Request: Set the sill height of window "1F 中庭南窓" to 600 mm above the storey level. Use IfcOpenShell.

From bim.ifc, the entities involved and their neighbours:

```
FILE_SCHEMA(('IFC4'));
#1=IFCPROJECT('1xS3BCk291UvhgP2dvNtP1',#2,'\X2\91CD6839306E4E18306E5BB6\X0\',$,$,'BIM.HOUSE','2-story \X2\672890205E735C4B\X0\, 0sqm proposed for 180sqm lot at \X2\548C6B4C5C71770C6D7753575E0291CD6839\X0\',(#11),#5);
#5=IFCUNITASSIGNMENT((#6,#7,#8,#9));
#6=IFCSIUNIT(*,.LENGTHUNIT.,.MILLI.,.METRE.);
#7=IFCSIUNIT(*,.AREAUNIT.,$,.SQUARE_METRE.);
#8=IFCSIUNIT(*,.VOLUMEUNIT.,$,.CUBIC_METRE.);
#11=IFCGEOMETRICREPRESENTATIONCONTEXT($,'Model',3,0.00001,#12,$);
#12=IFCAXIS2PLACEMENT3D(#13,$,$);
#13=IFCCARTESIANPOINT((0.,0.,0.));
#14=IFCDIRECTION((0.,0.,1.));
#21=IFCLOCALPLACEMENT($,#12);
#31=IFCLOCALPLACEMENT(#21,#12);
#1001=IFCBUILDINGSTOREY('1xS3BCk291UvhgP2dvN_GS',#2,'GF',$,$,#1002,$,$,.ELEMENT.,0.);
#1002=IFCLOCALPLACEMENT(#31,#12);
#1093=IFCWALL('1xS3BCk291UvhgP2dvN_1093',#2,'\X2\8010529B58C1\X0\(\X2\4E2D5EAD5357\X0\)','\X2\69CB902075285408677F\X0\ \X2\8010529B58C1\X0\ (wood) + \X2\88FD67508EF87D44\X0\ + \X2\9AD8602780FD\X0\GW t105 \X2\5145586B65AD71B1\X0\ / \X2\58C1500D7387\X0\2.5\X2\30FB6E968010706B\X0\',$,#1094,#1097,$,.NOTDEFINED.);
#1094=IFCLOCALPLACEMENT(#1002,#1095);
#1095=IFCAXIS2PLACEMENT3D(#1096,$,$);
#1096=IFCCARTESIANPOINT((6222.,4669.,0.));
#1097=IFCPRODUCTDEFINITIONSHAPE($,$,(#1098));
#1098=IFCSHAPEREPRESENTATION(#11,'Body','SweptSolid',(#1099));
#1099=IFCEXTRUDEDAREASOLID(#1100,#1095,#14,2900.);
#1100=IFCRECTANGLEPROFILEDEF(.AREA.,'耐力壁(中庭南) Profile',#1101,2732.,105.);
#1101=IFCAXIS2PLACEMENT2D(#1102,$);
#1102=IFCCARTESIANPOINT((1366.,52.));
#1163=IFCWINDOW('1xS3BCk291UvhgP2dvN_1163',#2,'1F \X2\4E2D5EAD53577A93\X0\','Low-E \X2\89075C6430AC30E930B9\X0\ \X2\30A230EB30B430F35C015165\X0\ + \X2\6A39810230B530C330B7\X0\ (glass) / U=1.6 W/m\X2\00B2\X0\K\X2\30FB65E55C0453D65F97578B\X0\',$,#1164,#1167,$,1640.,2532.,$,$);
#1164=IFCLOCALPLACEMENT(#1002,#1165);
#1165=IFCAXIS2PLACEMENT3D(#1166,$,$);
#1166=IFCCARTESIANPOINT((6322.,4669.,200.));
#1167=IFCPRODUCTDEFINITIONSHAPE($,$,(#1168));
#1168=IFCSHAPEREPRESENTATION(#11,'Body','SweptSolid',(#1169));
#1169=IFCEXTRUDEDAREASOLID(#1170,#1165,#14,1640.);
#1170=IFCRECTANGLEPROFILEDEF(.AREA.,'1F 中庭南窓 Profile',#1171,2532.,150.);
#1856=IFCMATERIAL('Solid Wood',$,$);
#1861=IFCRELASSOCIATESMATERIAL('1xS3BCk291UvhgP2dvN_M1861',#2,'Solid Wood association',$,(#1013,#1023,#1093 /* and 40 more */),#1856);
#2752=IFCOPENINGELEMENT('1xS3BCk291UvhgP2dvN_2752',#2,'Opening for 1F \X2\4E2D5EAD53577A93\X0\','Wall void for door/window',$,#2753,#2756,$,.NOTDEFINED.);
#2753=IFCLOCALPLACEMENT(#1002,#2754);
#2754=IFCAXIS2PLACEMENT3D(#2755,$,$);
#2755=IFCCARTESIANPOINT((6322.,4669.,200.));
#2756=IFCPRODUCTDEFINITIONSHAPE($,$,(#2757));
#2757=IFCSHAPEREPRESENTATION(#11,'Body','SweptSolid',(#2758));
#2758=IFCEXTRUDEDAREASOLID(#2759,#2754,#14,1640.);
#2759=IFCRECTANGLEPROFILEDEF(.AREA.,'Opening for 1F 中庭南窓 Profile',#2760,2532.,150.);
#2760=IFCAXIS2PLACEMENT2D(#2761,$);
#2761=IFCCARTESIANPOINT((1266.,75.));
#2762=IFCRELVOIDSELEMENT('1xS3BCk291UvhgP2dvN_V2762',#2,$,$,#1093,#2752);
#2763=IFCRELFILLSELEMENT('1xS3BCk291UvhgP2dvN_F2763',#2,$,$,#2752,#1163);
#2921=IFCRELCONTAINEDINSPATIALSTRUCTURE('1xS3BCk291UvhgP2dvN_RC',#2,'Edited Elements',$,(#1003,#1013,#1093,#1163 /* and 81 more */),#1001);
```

```python
import numpy as np
import ifcopenshell
import ifcopenshell.api.geometry
import ifcopenshell.geom
import ifcopenshell.util.element
import ifcopenshell.util.placement
import ifcopenshell.util.shape
import ifcopenshell.util.unit

model = ifcopenshell.open("bim.ifc")
unit_scale = ifcopenshell.util.unit.calculate_unit_scale(model)

window = model.by_guid("1xS3BCk291UvhgP2dvN_1163")
opening = window.FillsVoids[0].RelatingOpeningElement
storey = ifcopenshell.util.element.get_container(window, ifc_class="IfcBuildingStorey")
level = ifcopenshell.util.placement.get_local_placement(storey.ObjectPlacement)[2, 3]

# The opening's origin need not be at the sill, so measure its lowest point.
shape = ifcopenshell.geom.create_shape(ifcopenshell.geom.settings(), opening)
bottom = ifcopenshell.util.shape.get_shape_bottom_elevation(shape, shape.geometry) / unit_scale
dz = level + 0.6 / unit_scale - bottom

shift = np.array([0.0, 0.0, dz])
# The window is not placed relative to its opening, so move both.
for product in (opening, window):
    matrix = ifcopenshell.util.placement.get_local_placement(product.ObjectPlacement)
    matrix[:3, 3] += shift
    ifcopenshell.api.geometry.edit_object_placement(model, product=product, matrix=matrix, is_si=False)

print(f"moved by {dz * unit_scale:+.3f} m")

model.write("bim_v2.ifc")
```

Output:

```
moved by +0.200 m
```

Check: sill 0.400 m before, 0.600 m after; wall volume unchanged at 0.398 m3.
